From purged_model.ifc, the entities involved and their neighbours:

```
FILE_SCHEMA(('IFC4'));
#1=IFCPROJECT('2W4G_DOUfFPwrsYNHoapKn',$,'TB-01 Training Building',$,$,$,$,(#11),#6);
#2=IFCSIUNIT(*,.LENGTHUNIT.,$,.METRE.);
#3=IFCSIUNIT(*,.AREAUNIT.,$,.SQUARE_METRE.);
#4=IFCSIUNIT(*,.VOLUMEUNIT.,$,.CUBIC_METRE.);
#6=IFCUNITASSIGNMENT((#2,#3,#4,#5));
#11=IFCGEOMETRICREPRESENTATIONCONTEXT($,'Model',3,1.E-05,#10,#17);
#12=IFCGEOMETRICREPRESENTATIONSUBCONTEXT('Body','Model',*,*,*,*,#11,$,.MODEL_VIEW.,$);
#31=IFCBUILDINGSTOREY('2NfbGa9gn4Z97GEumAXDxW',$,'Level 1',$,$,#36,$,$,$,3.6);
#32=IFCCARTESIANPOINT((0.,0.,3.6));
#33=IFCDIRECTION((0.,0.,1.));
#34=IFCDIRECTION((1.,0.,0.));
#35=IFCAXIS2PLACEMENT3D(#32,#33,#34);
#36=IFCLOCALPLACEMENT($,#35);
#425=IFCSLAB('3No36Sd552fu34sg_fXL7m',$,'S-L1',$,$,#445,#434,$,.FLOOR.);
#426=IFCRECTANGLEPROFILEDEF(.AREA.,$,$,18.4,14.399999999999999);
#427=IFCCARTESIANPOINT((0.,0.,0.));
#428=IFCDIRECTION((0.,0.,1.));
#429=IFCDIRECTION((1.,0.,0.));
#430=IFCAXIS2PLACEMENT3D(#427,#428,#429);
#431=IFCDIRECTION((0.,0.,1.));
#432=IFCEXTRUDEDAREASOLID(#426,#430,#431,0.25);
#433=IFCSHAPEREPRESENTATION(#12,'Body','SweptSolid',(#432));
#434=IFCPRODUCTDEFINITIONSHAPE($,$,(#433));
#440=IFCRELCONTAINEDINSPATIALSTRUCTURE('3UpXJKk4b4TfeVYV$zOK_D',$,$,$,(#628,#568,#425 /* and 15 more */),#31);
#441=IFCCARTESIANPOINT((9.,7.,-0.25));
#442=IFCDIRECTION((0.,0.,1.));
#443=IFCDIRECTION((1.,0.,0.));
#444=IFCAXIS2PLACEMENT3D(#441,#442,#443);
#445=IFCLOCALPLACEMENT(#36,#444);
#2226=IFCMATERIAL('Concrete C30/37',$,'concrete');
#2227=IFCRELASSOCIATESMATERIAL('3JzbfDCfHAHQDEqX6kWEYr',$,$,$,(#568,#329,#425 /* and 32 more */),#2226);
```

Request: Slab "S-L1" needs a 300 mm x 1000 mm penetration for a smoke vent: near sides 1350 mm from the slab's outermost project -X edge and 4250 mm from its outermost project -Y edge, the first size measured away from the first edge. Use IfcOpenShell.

```python
import numpy as np
import ifcopenshell
import ifcopenshell.api.feature
import ifcopenshell.api.geometry
import ifcopenshell.api.root
import ifcopenshell.geom
import ifcopenshell.util.placement
import ifcopenshell.util.representation
import ifcopenshell.util.shape
import ifcopenshell.util.unit

model = ifcopenshell.open("purged_model.ifc")
unit_scale = ifcopenshell.util.unit.calculate_unit_scale(model)
settings = ifcopenshell.geom.settings()


def volume(element):
    """Net volume in cubic metres, openings subtracted."""
    shape = ifcopenshell.geom.create_shape(settings, element)
    return ifcopenshell.util.shape.get_volume(shape.geometry)


slab = model.by_guid("3No36Sd552fu34sg_fXL7m")
before = volume(slab)

# Extent in the slab's own axes, in metres. The edges named are its -X and -Y sides.
slab_shape = ifcopenshell.geom.create_shape(settings, slab)
vertices = ifcopenshell.util.shape.get_vertices(slab_shape.geometry)
x_min, y_min, bottom = vertices.min(axis=0)
top = vertices[:, 2].max()

opening = ifcopenshell.api.root.create_entity(model, ifc_class="IfcOpeningElement", name="Smoke vent opening", predefined_type="OPENING")
context = ifcopenshell.util.representation.get_context(model, "Model", "Body", "MODEL_VIEW")
width, depth = 0.3, 1
outline = [(0.0, 0.0), (width, 0.0), (width, depth), (0.0, depth), (0.0, 0.0)]
# Overshoot both faces by 50 mm so the cut is clean.
shape = ifcopenshell.api.geometry.add_slab_representation(
    model, context=context, depth=top - bottom + 0.1, polyline=outline
)
ifcopenshell.api.geometry.assign_representation(model, product=opening, representation=shape)

matrix = ifcopenshell.util.placement.get_local_placement(slab.ObjectPlacement)
matrix[:, 3] = matrix @ np.append(np.array([x_min + 1.35, y_min + 4.25, bottom - 0.05]) / unit_scale, 1.0)
ifcopenshell.api.geometry.edit_object_placement(model, product=opening, matrix=matrix, is_si=False)
ifcopenshell.api.feature.add_feature(model, feature=opening, element=slab)

after = volume(slab)

print(f"slab volume {before:.3f} -> {after:.3f} m3")

model.write("purged_model_v2.ifc")
```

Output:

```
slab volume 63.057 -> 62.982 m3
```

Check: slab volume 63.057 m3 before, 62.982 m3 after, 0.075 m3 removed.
